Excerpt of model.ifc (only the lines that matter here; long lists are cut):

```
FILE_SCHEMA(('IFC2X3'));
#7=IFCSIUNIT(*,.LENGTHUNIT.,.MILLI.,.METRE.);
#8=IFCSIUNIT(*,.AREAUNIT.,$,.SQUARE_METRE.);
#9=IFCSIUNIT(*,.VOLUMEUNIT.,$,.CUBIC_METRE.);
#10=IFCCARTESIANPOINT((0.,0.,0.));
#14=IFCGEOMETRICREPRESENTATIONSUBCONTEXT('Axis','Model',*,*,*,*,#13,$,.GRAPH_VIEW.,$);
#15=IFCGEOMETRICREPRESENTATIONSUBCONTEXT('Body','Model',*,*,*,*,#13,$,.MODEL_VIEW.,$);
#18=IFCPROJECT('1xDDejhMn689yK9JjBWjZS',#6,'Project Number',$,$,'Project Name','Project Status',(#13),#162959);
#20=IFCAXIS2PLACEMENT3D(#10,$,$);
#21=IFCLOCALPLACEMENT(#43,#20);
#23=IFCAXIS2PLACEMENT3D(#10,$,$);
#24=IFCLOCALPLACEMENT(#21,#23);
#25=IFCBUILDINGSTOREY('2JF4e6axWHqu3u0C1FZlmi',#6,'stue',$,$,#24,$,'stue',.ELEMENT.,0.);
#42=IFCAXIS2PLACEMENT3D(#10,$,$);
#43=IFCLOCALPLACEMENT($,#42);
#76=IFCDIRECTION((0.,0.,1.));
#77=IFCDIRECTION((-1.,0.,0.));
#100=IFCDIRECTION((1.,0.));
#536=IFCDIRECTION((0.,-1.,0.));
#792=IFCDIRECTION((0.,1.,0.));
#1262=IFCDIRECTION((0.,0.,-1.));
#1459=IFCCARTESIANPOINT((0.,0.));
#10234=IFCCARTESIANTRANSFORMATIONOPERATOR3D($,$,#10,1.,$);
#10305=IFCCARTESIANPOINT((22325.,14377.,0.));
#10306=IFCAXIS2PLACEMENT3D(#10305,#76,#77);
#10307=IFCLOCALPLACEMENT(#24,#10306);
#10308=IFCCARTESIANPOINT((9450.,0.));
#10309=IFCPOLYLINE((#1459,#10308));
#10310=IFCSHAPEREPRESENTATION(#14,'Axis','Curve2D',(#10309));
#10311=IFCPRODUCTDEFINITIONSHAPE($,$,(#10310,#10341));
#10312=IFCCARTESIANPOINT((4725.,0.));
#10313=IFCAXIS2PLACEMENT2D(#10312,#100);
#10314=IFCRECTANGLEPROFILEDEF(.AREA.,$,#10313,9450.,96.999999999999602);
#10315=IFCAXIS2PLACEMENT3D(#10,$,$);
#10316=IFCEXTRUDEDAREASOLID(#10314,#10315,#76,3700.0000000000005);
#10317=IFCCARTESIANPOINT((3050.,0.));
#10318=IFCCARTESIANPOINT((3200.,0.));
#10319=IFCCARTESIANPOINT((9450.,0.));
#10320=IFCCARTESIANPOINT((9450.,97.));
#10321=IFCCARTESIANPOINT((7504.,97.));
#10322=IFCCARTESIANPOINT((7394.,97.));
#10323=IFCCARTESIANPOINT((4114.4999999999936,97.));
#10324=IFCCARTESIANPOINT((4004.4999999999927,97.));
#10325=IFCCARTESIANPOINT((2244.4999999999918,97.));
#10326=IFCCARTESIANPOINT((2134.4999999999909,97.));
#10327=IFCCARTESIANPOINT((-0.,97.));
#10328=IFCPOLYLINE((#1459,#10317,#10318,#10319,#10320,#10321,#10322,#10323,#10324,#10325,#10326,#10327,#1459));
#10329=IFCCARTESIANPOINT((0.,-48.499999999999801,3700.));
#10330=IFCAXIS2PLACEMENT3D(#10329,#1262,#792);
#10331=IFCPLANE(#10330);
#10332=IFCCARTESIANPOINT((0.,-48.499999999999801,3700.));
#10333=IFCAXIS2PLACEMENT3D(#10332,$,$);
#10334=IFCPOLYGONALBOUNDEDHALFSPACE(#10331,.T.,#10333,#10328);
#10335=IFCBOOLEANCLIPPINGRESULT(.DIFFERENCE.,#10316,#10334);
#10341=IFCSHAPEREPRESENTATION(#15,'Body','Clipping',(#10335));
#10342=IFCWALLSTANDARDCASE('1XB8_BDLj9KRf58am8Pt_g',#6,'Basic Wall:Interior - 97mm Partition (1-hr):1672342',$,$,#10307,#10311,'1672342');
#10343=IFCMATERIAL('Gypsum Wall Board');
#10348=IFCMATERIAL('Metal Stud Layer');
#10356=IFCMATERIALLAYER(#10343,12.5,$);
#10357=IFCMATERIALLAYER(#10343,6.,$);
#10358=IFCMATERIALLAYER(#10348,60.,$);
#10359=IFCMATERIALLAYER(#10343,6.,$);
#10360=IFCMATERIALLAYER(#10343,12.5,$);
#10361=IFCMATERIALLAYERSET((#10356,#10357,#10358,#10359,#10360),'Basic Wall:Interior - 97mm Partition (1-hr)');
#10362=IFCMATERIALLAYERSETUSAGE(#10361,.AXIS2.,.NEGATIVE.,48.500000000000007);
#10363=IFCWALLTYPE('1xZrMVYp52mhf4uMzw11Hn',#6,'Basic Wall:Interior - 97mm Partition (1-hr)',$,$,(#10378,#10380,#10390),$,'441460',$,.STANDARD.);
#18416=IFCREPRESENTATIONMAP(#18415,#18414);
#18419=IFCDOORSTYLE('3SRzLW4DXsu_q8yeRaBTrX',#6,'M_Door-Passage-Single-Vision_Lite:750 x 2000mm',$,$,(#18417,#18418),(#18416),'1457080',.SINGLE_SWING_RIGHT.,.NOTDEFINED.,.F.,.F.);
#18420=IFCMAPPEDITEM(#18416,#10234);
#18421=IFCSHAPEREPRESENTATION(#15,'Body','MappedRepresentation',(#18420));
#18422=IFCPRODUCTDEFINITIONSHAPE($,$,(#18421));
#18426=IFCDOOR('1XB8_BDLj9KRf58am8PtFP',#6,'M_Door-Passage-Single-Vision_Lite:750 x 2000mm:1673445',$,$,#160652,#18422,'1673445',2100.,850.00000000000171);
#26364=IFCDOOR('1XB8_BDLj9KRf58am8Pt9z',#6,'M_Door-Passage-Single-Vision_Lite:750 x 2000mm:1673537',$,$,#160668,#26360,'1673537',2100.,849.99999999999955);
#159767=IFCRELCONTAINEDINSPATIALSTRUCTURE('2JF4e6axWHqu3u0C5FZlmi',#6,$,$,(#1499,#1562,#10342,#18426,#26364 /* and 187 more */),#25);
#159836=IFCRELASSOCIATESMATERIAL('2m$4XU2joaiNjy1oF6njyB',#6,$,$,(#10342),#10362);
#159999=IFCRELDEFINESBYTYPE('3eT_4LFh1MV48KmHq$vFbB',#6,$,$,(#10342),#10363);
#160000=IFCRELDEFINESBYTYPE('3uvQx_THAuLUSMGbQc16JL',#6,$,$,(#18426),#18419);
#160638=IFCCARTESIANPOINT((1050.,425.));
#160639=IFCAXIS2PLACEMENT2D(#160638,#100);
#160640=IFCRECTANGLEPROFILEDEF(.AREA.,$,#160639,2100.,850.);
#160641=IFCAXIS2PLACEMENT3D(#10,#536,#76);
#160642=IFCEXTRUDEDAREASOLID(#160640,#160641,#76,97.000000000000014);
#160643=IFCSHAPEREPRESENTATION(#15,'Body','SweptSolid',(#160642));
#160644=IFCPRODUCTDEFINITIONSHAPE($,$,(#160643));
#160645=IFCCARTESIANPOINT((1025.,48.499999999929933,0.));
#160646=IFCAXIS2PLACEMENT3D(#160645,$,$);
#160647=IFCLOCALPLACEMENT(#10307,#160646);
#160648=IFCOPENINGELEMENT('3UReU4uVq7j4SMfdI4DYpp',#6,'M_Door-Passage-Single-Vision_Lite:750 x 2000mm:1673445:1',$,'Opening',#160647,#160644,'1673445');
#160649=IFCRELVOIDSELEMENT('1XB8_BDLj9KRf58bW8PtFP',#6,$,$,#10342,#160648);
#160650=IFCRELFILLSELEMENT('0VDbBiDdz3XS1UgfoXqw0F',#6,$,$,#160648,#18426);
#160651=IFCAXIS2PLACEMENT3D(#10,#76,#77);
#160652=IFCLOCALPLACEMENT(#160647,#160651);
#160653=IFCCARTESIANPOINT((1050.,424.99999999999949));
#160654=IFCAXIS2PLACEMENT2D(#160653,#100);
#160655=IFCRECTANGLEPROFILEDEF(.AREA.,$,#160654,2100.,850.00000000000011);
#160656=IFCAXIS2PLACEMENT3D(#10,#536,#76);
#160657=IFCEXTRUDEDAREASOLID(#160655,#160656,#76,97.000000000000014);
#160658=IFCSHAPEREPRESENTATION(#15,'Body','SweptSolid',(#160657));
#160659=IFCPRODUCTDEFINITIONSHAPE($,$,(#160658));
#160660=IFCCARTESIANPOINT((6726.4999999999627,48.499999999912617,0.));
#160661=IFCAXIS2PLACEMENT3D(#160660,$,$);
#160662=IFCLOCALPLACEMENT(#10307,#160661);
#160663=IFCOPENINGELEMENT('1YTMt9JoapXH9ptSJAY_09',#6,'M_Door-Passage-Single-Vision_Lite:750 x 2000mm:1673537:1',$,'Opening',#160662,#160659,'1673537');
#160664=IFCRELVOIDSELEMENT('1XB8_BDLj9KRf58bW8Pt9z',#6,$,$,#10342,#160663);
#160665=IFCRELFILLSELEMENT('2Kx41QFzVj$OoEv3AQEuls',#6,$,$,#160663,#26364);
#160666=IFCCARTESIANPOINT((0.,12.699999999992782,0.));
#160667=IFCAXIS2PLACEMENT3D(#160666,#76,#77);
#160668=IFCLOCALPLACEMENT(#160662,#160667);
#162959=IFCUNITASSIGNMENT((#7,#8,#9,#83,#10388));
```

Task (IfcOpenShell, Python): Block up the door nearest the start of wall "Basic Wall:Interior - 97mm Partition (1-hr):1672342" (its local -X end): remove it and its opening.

```python
import ifcopenshell
import ifcopenshell.api.feature
import ifcopenshell.api.root
import ifcopenshell.geom
import ifcopenshell.util.shape

model = ifcopenshell.open("model.ifc")
settings = ifcopenshell.geom.settings()


def volume(element):
    """Net volume in cubic metres, openings subtracted."""
    shape = ifcopenshell.geom.create_shape(settings, element)
    return ifcopenshell.util.shape.get_volume(shape.geometry)


door = model.by_guid("1XB8_BDLj9KRf58am8PtFP")
opening = door.FillsVoids[0].RelatingOpeningElement
wall = opening.VoidsElements[0].RelatingBuildingElement
before = volume(wall)

ifcopenshell.api.root.remove_product(model, product=door)
ifcopenshell.api.feature.remove_feature(model, feature=opening)

after = volume(wall)

print(f"wall volume {before:.3f} -> {after:.3f} m3")

model.write("model_updated.ifc")
```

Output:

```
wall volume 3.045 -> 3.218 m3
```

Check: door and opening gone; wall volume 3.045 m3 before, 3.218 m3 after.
